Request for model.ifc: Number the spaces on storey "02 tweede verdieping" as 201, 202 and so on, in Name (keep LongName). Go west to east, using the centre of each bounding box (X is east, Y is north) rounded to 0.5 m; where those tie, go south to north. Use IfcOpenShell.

First a look at what the model holds.

```python
import ifcopenshell
import ifcopenshell.util.element
import ifcopenshell.util.placement

model = ifcopenshell.open("model.ifc")
print(model.schema)
storey = next(s for s in model.by_type("IfcBuildingStorey") if s.Name == "02 tweede verdieping")
spaces = [e for e in ifcopenshell.util.element.get_decomposition(storey) if e.is_a("IfcSpace")]
for e in sorted(spaces, key=lambda e: e.id()):
    origin = ifcopenshell.util.placement.get_local_placement(e.ObjectPlacement)[:3, 3]
    print(e.id(), e.Name, e.LongName, origin.round(2) + 0.0, sep=" | ")
```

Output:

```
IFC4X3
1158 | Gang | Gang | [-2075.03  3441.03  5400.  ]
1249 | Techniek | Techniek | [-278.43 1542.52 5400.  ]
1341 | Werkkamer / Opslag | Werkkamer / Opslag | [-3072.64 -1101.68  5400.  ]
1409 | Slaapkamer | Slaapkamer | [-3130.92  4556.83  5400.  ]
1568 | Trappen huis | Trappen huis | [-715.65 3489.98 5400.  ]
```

```python
import ifcopenshell
import ifcopenshell.geom
import ifcopenshell.util.element
import ifcopenshell.util.shape

model = ifcopenshell.open("model.ifc")
settings = ifcopenshell.geom.settings()
settings.set("use-world-coords", True)


def centre(element):
    shape = ifcopenshell.geom.create_shape(settings, element)
    return ifcopenshell.util.shape.get_bbox_centroid(shape.geometry)


storey = next(s for s in model.by_type("IfcBuildingStorey") if s.Name == "02 tweede verdieping")
spaces = [e for e in ifcopenshell.util.element.get_decomposition(storey) if e.is_a("IfcSpace")]

# Insertion points can sit at a corner or the storey origin, so sort by the geometry (in metres).
centres = {e: centre(e) for e in spaces}
spaces.sort(key=lambda e: (round(centres[e][0] / 0.5), centres[e][1]))

for i, e in enumerate(spaces, start=1):
    number = f"2{i:02d}"
    e.Name = number
    print(e.id(), number)

model.write("model_rev.ifc")
```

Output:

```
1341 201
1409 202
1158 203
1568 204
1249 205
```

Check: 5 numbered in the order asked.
